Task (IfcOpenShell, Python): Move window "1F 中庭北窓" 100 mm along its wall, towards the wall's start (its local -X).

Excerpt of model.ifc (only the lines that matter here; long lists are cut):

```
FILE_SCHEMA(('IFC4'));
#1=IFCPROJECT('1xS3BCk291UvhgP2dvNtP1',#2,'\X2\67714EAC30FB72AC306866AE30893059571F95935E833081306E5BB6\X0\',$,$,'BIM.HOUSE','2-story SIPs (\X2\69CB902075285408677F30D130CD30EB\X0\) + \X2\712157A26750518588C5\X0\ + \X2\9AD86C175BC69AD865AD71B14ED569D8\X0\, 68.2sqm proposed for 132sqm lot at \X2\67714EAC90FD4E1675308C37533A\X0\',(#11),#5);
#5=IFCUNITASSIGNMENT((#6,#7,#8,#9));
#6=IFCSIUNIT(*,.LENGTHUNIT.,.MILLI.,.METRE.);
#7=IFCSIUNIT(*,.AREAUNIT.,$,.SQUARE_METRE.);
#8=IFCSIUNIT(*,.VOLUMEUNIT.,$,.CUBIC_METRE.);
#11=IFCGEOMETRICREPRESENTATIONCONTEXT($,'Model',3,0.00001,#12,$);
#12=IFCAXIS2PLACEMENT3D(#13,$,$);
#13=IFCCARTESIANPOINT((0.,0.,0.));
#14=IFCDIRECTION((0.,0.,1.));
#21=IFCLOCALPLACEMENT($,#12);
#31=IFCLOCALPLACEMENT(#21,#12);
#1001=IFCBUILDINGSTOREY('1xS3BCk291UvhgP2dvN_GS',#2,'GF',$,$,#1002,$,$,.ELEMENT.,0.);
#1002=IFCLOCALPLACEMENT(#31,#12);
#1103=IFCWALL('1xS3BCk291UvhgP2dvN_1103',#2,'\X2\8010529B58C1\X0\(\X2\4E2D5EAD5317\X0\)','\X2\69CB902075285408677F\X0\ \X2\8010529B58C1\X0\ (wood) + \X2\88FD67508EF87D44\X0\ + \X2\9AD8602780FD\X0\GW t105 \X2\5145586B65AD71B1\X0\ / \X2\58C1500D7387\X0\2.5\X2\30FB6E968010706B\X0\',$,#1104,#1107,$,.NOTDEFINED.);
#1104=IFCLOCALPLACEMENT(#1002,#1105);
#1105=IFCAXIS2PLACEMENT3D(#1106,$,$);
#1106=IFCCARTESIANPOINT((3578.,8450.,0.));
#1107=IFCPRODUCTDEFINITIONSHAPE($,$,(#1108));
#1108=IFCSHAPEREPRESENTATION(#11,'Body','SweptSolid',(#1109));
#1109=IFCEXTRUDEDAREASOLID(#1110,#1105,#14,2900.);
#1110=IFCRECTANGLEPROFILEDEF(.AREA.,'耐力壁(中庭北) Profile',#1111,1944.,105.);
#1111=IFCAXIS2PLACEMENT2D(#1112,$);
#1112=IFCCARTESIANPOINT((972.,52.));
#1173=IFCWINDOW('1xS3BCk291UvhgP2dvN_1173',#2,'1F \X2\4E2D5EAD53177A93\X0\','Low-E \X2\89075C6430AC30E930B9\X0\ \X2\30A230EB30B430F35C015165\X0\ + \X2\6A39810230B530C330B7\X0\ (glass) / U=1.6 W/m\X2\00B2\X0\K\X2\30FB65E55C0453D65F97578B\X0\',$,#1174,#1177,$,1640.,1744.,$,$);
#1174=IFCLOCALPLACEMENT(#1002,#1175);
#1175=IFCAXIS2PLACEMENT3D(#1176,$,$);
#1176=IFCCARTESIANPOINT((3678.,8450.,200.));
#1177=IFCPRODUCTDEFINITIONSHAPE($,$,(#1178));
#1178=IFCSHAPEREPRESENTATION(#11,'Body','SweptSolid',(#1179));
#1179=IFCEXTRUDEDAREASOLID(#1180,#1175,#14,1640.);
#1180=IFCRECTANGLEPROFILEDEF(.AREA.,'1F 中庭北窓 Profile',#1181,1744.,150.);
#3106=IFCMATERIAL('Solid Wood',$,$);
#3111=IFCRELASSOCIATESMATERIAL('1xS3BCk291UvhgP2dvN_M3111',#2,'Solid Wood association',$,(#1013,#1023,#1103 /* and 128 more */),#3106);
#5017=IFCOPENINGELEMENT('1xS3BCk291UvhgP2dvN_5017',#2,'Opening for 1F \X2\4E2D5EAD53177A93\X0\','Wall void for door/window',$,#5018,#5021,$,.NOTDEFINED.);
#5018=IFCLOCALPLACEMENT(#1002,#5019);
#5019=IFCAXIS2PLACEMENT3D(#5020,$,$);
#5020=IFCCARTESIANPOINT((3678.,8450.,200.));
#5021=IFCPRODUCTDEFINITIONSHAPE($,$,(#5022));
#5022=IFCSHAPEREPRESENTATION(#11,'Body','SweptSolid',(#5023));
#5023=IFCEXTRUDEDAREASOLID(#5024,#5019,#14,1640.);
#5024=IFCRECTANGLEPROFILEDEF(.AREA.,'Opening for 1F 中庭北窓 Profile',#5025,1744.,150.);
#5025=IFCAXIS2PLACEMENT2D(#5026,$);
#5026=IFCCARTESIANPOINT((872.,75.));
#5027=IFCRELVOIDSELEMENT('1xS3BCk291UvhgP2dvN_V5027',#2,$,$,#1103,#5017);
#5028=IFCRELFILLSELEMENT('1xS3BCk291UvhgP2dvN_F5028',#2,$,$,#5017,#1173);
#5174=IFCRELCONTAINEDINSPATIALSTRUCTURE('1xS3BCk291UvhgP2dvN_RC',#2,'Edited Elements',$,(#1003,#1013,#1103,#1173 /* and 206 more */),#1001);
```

```python
import ifcopenshell
import ifcopenshell.api.geometry
import ifcopenshell.util.placement
import ifcopenshell.util.unit

model = ifcopenshell.open("model.ifc")
unit_scale = ifcopenshell.util.unit.calculate_unit_scale(model)

window = model.by_guid("1xS3BCk291UvhgP2dvN_1173")
opening = window.FillsVoids[0].RelatingOpeningElement
wall = opening.VoidsElements[0].RelatingBuildingElement

wall_matrix = ifcopenshell.util.placement.get_local_placement(wall.ObjectPlacement)
shift = wall_matrix[:3, 0] * -0.1 / unit_scale
before = ifcopenshell.util.placement.get_local_placement(window.ObjectPlacement)[:3, 3].copy()

# The window is not placed relative to its opening, so move both.
for product in (opening, window):
    matrix = ifcopenshell.util.placement.get_local_placement(product.ObjectPlacement)
    matrix[:3, 3] += shift
    ifcopenshell.api.geometry.edit_object_placement(model, product=product, matrix=matrix, is_si=False)

after = ifcopenshell.util.placement.get_local_placement(window.ObjectPlacement)[:3, 3]
print("window moved by", (after - before).round(3) + 0.0)

model.write("model_updated.ifc")
```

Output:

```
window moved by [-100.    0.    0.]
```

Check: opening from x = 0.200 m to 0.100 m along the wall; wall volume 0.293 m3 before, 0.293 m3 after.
